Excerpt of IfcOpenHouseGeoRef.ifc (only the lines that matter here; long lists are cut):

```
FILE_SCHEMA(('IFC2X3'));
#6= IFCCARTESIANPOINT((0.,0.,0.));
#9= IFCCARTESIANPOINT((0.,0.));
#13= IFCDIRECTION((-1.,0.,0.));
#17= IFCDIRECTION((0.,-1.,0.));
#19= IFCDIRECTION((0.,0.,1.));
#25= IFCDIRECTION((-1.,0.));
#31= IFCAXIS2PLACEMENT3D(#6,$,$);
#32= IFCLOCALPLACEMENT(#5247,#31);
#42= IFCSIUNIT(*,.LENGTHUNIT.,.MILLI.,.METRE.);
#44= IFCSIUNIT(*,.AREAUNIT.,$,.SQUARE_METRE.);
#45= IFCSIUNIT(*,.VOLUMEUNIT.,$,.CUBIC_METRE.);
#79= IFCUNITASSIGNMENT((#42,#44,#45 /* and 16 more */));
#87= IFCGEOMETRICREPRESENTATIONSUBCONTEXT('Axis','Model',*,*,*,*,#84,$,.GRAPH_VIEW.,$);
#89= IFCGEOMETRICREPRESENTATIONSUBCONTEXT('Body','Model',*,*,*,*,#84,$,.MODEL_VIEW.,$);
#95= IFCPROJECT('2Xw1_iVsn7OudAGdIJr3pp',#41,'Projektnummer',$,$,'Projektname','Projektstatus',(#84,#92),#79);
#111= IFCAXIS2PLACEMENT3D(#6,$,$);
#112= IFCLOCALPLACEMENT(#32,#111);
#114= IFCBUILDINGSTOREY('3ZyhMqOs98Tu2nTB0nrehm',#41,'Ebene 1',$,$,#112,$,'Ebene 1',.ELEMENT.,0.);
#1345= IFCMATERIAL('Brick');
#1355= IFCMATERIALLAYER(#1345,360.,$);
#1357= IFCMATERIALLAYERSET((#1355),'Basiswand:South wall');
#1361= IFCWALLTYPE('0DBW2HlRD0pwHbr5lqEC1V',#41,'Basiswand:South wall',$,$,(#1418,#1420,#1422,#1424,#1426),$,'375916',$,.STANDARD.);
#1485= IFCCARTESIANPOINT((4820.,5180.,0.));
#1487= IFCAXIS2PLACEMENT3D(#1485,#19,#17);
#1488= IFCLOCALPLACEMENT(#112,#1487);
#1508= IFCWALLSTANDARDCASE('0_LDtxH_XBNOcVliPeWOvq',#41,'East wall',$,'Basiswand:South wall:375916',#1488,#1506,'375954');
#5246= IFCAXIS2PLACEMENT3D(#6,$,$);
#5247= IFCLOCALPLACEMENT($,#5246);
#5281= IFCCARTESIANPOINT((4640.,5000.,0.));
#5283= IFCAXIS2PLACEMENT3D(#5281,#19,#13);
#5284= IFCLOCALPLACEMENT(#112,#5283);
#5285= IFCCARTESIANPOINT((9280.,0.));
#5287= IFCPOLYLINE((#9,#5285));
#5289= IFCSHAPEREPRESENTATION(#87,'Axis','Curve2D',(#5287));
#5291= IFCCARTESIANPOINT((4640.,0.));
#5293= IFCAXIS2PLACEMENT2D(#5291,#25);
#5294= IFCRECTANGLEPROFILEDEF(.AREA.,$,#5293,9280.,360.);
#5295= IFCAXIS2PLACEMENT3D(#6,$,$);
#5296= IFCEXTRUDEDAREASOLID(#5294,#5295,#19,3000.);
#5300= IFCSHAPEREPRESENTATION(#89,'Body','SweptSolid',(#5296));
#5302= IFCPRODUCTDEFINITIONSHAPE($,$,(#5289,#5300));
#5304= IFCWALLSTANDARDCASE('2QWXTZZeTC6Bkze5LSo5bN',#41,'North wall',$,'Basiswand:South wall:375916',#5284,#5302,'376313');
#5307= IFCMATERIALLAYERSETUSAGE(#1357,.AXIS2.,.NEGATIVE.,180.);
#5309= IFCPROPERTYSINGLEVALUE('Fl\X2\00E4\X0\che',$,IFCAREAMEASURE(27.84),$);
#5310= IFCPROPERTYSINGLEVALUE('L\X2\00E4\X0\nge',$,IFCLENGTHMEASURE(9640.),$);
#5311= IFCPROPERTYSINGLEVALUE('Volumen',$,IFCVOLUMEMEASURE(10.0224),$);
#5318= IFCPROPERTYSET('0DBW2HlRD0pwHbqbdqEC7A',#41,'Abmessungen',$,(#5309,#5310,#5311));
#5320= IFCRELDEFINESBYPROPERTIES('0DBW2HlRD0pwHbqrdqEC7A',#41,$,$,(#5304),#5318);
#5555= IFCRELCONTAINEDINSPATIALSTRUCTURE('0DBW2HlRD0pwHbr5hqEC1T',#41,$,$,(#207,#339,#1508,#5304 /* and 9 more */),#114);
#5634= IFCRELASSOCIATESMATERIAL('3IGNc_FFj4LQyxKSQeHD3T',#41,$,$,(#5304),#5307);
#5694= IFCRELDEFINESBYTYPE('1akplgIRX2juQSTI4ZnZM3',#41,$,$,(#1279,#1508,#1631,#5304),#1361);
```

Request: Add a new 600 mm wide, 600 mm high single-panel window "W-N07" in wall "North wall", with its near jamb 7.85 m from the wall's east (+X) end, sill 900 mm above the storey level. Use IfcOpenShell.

```python
import numpy as np
import ifcopenshell
import ifcopenshell.api.feature
import ifcopenshell.api.geometry
import ifcopenshell.api.pset
import ifcopenshell.api.root
import ifcopenshell.api.spatial
import ifcopenshell.api.type
import ifcopenshell.geom
import ifcopenshell.util.element
import ifcopenshell.util.placement
import ifcopenshell.util.representation
import ifcopenshell.util.shape
import ifcopenshell.util.unit

model = ifcopenshell.open("IfcOpenHouseGeoRef.ifc")
unit_scale = ifcopenshell.util.unit.calculate_unit_scale(model)
area_scale = ifcopenshell.util.unit.calculate_unit_scale(model, "AREAUNIT")
volume_scale = ifcopenshell.util.unit.calculate_unit_scale(model, "VOLUMEUNIT")
settings = ifcopenshell.geom.settings()


def volume(element):
    """Net volume in cubic metres, openings subtracted."""
    shape = ifcopenshell.geom.create_shape(settings, element)
    return ifcopenshell.util.shape.get_volume(shape.geometry)


wall = model.by_guid("2QWXTZZeTC6Bkze5LSo5bN")
storey = ifcopenshell.util.element.get_container(wall, ifc_class="IfcBuildingStorey")
context = ifcopenshell.util.representation.get_context(model, "Model", "Body", "MODEL_VIEW")
before = volume(wall)

width, height, from_end, sill = 0.6, 0.6, 7.85, 0.9  # metres

# The wall runs along its own X axis, and the end named is its -X end.
wall_shape = ifcopenshell.geom.create_shape(settings, wall)
x, y, z = ifcopenshell.util.shape.get_vertices(wall_shape.geometry).T
start = x.min() + from_end
face, thickness = float(y.min()), float(y.max() - y.min())
wall_matrix = ifcopenshell.util.placement.get_local_placement(wall.ObjectPlacement)
level = ifcopenshell.util.placement.get_local_placement(storey.ObjectPlacement)[2, 3]


def in_wall(x, y):
    """Placement at x, y metres in the wall's axes, at sill height."""
    matrix = wall_matrix.copy()
    matrix[:, 3] = wall_matrix @ np.array([x / unit_scale, y / unit_scale, 0.0, 1.0])
    matrix[2, 3] = level + sill / unit_scale
    return matrix


# Opening: a box that overshoots both wall faces by 50 mm.
opening = ifcopenshell.api.root.create_entity(model, ifc_class="IfcOpeningElement")
box = ifcopenshell.api.geometry.add_wall_representation(
    model, context=context, length=width, height=height, thickness=thickness + 0.1
)
ifcopenshell.api.geometry.assign_representation(model, product=opening, representation=box)
ifcopenshell.api.geometry.edit_object_placement(model, product=opening, matrix=in_wall(start, face - 0.05), is_si=False)
ifcopenshell.api.feature.add_feature(model, feature=opening, element=wall)

window = ifcopenshell.api.root.create_entity(model, ifc_class="IfcWindow", name="W-N07")
window.OverallWidth, window.OverallHeight = width / unit_scale, height / unit_scale
body = ifcopenshell.api.geometry.add_window_representation(
    model,
    context=context,
    overall_width=window.OverallWidth,
    overall_height=window.OverallHeight,
    partition_type="SINGLE_PANEL",
)
ifcopenshell.api.geometry.assign_representation(model, product=window, representation=body)
ifcopenshell.api.spatial.assign_container(model, products=[window], relating_structure=storey)
fills = ifcopenshell.api.feature.add_filling(model, opening=opening, element=window)
fills.OwnerHistory = window.OwnerHistory  # required in IFC2X3

# IFC2X3 keeps the operation on the window style.
style = ifcopenshell.api.root.create_entity(model, ifc_class="IfcWindowStyle", name="W-N07")
style.OperationType, style.ConstructionType = "SINGLE_PANEL", "NOTDEFINED"
style.ParameterTakesPrecedence = style.Sizeable = False
ifcopenshell.api.type.assign_type(model, related_objects=[window], relating_type=style)

# Centre the window in the wall's thickness.
ifcopenshell.api.geometry.edit_object_placement(model, product=window, matrix=in_wall(start, face), is_si=False)
window_shape = ifcopenshell.geom.create_shape(settings, window)
depth = ifcopenshell.util.shape.get_vertices(window_shape.geometry)[:, 1]
offset = face + thickness / 2 - (depth.min() + depth.max()) / 2
ifcopenshell.api.geometry.edit_object_placement(model, product=window, matrix=in_wall(start, offset), is_si=False)

after = volume(wall)

# Update the wall's stored quantities.
pset = model.by_id(ifcopenshell.util.element.get_pset(wall, "Abmessungen", should_inherit=False)["id"])
ifcopenshell.api.pset.edit_pset(model, pset=pset, properties={
    "Fläche": model.create_entity("IfcAreaMeasure", after / thickness / area_scale),
    "Volumen": model.create_entity("IfcVolumeMeasure", after / volume_scale),
})

print(f"wall volume {before:.3f} -> {after:.3f} m3")

model.write("IfcOpenHouseGeoRef-out.ifc")
```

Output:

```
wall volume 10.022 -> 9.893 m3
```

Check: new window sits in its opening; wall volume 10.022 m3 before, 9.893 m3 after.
